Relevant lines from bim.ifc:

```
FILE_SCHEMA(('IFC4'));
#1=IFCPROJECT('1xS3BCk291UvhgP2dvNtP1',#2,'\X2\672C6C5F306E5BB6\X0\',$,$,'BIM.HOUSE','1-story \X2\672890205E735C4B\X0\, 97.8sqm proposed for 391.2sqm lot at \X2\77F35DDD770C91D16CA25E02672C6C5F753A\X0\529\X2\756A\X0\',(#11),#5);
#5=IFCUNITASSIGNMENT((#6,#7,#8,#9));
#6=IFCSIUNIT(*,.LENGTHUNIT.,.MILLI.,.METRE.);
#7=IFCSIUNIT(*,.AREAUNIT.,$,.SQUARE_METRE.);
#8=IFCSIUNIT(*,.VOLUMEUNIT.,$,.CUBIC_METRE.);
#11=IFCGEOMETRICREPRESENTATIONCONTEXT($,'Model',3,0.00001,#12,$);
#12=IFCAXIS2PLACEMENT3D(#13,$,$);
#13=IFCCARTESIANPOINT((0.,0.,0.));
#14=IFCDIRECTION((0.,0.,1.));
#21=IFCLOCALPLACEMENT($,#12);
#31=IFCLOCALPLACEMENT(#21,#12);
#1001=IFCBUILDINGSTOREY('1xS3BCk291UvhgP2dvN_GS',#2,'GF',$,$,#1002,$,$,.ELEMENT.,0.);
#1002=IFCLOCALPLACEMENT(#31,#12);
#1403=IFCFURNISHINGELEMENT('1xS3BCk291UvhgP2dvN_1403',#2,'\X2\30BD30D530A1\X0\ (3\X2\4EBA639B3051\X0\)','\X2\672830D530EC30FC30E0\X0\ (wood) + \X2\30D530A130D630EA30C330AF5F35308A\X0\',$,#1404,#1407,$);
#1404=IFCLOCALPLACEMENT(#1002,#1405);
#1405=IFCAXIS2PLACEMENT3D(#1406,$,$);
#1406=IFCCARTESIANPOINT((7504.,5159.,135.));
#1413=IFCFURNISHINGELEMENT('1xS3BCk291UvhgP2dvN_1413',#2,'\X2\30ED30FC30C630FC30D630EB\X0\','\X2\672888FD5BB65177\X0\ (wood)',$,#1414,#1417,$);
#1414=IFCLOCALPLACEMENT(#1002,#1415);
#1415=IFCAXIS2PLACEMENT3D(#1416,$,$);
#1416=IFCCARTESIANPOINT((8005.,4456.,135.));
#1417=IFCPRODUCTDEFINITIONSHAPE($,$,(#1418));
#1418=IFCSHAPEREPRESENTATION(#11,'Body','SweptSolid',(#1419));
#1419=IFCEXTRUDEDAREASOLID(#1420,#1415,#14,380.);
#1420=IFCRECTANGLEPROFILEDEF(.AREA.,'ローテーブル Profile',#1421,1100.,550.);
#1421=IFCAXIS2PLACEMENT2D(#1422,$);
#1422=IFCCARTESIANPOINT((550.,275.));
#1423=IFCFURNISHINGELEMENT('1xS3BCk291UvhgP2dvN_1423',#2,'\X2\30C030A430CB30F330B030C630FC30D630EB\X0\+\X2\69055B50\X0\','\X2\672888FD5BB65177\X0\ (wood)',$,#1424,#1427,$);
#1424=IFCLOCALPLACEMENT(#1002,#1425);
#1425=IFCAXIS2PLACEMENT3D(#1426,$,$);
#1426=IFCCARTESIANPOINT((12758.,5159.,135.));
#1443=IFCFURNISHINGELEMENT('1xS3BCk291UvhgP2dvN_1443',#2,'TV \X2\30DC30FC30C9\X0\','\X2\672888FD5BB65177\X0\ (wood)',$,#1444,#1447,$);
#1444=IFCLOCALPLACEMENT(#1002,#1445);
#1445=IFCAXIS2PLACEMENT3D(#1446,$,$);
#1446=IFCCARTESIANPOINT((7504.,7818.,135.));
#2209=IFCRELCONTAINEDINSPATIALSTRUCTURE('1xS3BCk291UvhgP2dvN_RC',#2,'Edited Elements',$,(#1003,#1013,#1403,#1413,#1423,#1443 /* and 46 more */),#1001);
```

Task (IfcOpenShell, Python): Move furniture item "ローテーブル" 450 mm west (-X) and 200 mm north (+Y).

```python
import ifcopenshell
import ifcopenshell.api.geometry
import ifcopenshell.util.placement
import ifcopenshell.util.unit

model = ifcopenshell.open("bim.ifc")
unit_scale = ifcopenshell.util.unit.calculate_unit_scale(model)

item = model.by_guid("1xS3BCk291UvhgP2dvN_1413")
matrix = ifcopenshell.util.placement.get_local_placement(item.ObjectPlacement)
matrix[0, 3] -= 0.45 / unit_scale
matrix[1, 3] += 0.2 / unit_scale
ifcopenshell.api.geometry.edit_object_placement(model, product=item, matrix=matrix, is_si=False)

print(ifcopenshell.util.placement.get_local_placement(item.ObjectPlacement).round(3) + 0.0)

model.write("bim_rev.ifc")
```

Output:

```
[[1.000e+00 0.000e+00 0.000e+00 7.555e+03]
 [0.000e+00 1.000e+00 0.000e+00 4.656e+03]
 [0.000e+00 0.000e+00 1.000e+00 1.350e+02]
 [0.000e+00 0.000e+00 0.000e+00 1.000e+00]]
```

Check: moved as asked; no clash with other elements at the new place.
